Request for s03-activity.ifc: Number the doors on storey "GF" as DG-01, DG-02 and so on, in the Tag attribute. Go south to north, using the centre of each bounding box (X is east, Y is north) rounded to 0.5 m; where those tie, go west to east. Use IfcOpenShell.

First a look at what the model holds.

```python
import ifcopenshell
import ifcopenshell.util.element
import ifcopenshell.util.placement

model = ifcopenshell.open("s03-activity.ifc")
print(model.schema)
storey = next(s for s in model.by_type("IfcBuildingStorey") if s.Name == "GF")
doors = [e for e in ifcopenshell.util.element.get_decomposition(storey) if e.is_a("IfcDoor")]
for e in sorted(doors, key=lambda e: e.id()):
    origin = ifcopenshell.util.placement.get_local_placement(e.ObjectPlacement)[:3, 3]
    print(e.id(), e.Tag, e.Name, origin.round(2) + 0.0, sep=" | ")
```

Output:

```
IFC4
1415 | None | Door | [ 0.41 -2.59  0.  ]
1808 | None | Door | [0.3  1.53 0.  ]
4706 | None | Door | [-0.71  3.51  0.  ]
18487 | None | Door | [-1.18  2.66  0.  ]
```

```python
import ifcopenshell
import ifcopenshell.geom
import ifcopenshell.util.element
import ifcopenshell.util.shape

model = ifcopenshell.open("s03-activity.ifc")
settings = ifcopenshell.geom.settings()
settings.set("use-world-coords", True)


def centre(element):
    shape = ifcopenshell.geom.create_shape(settings, element)
    return ifcopenshell.util.shape.get_bbox_centroid(shape.geometry)


storey = next(s for s in model.by_type("IfcBuildingStorey") if s.Name == "GF")
doors = [e for e in ifcopenshell.util.element.get_decomposition(storey) if e.is_a("IfcDoor")]

# Insertion points can sit at a corner or the storey origin, so sort by the geometry (in metres).
centres = {e: centre(e) for e in doors}
doors.sort(key=lambda e: (round(centres[e][1] / 0.5), centres[e][0]))

for i, e in enumerate(doors, start=1):
    number = f"DG-{i:02d}"
    e.Tag = number
    print(e.id(), number)

model.write("s03-activity_updated.ifc")
```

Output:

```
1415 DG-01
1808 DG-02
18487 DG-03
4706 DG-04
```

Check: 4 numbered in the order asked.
